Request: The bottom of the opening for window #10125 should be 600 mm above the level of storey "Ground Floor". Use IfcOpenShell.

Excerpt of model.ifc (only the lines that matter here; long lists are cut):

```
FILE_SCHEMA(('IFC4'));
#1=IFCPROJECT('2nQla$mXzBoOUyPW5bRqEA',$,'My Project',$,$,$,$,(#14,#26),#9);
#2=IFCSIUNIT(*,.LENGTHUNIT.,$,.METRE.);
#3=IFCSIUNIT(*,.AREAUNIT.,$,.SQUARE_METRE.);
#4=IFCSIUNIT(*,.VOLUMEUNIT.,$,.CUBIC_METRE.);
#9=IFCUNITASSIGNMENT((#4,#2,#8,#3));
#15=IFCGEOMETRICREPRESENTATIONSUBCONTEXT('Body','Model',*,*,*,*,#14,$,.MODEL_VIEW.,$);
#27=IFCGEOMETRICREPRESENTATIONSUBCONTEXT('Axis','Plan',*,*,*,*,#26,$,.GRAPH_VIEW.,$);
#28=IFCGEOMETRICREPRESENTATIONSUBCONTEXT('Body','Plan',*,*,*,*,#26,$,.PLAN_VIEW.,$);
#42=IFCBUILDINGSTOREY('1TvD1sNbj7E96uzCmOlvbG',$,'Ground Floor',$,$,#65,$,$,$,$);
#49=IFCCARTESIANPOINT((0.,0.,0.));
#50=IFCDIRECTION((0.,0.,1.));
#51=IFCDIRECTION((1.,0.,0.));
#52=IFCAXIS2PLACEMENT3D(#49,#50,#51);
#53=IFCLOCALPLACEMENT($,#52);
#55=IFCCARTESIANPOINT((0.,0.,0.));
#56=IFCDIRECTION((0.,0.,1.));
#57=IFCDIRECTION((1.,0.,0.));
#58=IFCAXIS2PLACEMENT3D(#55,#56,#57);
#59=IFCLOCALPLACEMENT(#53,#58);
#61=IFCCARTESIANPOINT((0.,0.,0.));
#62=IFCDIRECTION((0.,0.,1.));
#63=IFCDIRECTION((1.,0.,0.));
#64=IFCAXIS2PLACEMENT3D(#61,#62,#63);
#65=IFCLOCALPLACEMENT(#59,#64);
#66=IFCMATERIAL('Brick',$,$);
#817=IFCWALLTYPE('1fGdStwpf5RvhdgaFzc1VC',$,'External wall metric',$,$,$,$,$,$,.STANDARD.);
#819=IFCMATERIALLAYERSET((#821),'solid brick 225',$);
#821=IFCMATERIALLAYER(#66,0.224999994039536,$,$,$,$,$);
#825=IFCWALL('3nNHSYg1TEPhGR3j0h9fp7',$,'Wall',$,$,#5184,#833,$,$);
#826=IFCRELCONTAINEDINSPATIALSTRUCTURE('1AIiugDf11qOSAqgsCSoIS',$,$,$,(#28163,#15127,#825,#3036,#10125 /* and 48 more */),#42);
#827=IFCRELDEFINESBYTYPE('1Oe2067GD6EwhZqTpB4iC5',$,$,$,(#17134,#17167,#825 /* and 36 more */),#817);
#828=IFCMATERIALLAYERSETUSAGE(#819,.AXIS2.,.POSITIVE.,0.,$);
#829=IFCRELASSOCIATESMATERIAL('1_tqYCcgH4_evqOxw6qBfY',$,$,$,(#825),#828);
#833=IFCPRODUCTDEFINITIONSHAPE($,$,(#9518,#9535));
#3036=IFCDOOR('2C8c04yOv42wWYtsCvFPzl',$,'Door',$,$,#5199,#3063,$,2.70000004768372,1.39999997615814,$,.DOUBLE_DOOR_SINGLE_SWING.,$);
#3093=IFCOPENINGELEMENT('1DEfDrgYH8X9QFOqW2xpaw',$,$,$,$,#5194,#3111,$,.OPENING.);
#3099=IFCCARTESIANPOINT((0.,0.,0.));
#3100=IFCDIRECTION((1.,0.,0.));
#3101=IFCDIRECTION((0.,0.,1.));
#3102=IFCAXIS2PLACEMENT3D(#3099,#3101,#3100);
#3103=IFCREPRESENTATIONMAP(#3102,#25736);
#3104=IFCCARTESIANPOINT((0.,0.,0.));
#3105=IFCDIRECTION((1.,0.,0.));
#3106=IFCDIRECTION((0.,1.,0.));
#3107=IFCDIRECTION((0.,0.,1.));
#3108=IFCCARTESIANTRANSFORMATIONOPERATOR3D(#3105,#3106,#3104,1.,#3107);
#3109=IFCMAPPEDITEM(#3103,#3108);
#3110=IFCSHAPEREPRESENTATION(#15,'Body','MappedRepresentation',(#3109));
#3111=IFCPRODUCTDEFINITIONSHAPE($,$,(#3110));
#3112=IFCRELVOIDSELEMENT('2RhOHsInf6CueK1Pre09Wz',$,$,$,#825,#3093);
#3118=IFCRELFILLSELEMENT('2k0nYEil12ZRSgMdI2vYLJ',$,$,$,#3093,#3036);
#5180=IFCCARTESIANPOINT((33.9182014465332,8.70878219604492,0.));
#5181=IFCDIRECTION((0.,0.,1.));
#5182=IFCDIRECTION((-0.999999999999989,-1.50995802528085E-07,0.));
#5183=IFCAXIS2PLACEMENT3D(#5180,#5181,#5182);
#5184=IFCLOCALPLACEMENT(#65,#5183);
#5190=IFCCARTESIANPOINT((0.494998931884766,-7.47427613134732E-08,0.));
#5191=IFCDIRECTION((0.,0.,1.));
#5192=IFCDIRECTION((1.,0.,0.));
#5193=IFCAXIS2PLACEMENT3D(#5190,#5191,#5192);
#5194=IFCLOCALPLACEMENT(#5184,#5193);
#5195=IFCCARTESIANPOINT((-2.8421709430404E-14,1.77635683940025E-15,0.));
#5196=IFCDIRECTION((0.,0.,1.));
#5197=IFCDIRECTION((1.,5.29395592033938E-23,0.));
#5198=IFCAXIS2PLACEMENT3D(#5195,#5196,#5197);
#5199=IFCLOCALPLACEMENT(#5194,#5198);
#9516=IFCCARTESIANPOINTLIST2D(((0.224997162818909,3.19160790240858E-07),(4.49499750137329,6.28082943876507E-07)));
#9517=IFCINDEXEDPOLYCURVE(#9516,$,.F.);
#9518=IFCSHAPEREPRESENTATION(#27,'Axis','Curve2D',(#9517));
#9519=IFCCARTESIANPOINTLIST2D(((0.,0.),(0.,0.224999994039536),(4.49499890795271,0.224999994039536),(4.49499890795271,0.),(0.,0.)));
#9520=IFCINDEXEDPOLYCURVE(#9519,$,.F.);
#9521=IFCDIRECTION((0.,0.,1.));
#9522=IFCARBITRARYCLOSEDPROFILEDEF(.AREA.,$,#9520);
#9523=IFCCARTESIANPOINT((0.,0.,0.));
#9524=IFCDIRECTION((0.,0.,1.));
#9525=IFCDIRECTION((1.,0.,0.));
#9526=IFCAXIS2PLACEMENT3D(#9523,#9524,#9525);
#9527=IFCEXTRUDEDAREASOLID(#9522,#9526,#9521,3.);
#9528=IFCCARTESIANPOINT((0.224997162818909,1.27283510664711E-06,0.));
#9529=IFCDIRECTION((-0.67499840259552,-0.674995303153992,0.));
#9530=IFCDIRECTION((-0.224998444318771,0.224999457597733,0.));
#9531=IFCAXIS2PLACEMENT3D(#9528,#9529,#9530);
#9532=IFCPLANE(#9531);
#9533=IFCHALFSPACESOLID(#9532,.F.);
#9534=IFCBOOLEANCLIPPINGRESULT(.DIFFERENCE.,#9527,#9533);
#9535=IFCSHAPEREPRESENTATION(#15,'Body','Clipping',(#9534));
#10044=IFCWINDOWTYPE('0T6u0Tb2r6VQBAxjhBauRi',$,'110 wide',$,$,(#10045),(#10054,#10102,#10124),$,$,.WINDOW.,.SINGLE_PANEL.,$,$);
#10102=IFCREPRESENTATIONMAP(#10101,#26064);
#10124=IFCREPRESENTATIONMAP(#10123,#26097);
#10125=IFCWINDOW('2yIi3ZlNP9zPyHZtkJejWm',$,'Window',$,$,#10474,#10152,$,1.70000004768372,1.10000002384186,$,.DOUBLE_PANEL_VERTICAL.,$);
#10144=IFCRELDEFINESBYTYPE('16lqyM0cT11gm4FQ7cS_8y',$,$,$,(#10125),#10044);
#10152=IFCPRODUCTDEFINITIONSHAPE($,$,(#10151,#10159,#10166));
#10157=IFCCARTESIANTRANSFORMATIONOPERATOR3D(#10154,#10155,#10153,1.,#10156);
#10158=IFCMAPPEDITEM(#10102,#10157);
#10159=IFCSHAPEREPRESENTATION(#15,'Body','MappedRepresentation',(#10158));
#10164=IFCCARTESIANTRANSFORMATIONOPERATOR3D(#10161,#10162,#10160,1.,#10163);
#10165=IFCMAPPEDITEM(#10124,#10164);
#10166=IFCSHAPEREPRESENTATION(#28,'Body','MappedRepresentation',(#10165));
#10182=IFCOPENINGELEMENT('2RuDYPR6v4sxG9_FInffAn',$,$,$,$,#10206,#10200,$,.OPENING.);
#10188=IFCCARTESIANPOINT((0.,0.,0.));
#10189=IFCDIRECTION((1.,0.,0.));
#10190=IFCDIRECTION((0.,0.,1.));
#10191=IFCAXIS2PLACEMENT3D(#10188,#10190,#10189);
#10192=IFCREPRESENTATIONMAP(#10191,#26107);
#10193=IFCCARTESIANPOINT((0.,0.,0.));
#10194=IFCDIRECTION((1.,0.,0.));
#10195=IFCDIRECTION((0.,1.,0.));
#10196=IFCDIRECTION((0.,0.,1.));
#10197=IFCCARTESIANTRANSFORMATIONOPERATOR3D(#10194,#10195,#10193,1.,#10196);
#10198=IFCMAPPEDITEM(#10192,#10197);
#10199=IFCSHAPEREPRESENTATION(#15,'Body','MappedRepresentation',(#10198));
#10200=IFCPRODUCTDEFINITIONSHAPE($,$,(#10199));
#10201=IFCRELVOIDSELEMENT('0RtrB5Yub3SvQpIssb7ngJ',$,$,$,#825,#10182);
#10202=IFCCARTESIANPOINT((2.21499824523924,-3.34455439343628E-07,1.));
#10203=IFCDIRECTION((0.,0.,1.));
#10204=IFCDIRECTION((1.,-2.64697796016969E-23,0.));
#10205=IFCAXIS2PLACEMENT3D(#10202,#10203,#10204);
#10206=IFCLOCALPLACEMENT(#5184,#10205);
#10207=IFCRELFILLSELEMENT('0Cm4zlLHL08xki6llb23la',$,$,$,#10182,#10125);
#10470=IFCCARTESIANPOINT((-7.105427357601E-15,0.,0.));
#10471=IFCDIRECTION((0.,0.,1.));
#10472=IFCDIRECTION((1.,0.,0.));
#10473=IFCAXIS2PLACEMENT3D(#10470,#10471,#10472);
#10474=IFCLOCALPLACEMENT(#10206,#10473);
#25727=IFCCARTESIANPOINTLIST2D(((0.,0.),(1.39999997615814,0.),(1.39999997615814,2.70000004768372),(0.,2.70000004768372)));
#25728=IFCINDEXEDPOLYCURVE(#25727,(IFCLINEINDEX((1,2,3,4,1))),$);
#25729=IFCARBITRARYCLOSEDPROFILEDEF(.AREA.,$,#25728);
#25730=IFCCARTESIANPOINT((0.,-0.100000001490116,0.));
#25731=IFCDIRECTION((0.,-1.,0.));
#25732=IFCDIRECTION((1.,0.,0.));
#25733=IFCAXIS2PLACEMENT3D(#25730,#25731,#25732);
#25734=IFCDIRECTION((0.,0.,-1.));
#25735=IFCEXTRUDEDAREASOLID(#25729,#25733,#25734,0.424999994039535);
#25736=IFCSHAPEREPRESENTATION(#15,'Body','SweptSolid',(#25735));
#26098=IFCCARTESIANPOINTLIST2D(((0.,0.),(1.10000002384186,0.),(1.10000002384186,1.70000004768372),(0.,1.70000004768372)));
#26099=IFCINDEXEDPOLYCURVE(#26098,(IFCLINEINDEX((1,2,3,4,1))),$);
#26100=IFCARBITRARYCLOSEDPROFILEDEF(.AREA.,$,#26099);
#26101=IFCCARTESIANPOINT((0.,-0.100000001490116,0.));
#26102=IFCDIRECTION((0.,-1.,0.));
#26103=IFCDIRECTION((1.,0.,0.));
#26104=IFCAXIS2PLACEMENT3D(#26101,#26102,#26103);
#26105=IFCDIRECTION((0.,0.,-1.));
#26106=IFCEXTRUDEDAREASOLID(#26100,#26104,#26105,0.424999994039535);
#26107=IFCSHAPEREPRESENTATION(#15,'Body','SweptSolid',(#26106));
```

```python
import numpy as np
import ifcopenshell
import ifcopenshell.api.geometry
import ifcopenshell.geom
import ifcopenshell.util.element
import ifcopenshell.util.placement
import ifcopenshell.util.shape
import ifcopenshell.util.unit

model = ifcopenshell.open("model.ifc")
unit_scale = ifcopenshell.util.unit.calculate_unit_scale(model)

window = model.by_guid("2yIi3ZlNP9zPyHZtkJejWm")
opening = window.FillsVoids[0].RelatingOpeningElement
storey = ifcopenshell.util.element.get_container(window, ifc_class="IfcBuildingStorey")
level = ifcopenshell.util.placement.get_local_placement(storey.ObjectPlacement)[2, 3]

# The opening's origin need not be at the sill, so measure its lowest point.
shape = ifcopenshell.geom.create_shape(ifcopenshell.geom.settings(), opening)
bottom = ifcopenshell.util.shape.get_shape_bottom_elevation(shape, shape.geometry) / unit_scale
dz = level + 0.6 - bottom

shift = np.array([0.0, 0.0, dz])
# The window is placed relative to its opening, so it follows when the opening moves.
matrix = ifcopenshell.util.placement.get_local_placement(opening.ObjectPlacement)
matrix[:3, 3] += shift
ifcopenshell.api.geometry.edit_object_placement(
    model, product=opening, matrix=matrix, is_si=False, should_transform_children=True
)

print(f"moved by {dz * unit_scale:+.3f} m")

model.write("model_rev.ifc")
```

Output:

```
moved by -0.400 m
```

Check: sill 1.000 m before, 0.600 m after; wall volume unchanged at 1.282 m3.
